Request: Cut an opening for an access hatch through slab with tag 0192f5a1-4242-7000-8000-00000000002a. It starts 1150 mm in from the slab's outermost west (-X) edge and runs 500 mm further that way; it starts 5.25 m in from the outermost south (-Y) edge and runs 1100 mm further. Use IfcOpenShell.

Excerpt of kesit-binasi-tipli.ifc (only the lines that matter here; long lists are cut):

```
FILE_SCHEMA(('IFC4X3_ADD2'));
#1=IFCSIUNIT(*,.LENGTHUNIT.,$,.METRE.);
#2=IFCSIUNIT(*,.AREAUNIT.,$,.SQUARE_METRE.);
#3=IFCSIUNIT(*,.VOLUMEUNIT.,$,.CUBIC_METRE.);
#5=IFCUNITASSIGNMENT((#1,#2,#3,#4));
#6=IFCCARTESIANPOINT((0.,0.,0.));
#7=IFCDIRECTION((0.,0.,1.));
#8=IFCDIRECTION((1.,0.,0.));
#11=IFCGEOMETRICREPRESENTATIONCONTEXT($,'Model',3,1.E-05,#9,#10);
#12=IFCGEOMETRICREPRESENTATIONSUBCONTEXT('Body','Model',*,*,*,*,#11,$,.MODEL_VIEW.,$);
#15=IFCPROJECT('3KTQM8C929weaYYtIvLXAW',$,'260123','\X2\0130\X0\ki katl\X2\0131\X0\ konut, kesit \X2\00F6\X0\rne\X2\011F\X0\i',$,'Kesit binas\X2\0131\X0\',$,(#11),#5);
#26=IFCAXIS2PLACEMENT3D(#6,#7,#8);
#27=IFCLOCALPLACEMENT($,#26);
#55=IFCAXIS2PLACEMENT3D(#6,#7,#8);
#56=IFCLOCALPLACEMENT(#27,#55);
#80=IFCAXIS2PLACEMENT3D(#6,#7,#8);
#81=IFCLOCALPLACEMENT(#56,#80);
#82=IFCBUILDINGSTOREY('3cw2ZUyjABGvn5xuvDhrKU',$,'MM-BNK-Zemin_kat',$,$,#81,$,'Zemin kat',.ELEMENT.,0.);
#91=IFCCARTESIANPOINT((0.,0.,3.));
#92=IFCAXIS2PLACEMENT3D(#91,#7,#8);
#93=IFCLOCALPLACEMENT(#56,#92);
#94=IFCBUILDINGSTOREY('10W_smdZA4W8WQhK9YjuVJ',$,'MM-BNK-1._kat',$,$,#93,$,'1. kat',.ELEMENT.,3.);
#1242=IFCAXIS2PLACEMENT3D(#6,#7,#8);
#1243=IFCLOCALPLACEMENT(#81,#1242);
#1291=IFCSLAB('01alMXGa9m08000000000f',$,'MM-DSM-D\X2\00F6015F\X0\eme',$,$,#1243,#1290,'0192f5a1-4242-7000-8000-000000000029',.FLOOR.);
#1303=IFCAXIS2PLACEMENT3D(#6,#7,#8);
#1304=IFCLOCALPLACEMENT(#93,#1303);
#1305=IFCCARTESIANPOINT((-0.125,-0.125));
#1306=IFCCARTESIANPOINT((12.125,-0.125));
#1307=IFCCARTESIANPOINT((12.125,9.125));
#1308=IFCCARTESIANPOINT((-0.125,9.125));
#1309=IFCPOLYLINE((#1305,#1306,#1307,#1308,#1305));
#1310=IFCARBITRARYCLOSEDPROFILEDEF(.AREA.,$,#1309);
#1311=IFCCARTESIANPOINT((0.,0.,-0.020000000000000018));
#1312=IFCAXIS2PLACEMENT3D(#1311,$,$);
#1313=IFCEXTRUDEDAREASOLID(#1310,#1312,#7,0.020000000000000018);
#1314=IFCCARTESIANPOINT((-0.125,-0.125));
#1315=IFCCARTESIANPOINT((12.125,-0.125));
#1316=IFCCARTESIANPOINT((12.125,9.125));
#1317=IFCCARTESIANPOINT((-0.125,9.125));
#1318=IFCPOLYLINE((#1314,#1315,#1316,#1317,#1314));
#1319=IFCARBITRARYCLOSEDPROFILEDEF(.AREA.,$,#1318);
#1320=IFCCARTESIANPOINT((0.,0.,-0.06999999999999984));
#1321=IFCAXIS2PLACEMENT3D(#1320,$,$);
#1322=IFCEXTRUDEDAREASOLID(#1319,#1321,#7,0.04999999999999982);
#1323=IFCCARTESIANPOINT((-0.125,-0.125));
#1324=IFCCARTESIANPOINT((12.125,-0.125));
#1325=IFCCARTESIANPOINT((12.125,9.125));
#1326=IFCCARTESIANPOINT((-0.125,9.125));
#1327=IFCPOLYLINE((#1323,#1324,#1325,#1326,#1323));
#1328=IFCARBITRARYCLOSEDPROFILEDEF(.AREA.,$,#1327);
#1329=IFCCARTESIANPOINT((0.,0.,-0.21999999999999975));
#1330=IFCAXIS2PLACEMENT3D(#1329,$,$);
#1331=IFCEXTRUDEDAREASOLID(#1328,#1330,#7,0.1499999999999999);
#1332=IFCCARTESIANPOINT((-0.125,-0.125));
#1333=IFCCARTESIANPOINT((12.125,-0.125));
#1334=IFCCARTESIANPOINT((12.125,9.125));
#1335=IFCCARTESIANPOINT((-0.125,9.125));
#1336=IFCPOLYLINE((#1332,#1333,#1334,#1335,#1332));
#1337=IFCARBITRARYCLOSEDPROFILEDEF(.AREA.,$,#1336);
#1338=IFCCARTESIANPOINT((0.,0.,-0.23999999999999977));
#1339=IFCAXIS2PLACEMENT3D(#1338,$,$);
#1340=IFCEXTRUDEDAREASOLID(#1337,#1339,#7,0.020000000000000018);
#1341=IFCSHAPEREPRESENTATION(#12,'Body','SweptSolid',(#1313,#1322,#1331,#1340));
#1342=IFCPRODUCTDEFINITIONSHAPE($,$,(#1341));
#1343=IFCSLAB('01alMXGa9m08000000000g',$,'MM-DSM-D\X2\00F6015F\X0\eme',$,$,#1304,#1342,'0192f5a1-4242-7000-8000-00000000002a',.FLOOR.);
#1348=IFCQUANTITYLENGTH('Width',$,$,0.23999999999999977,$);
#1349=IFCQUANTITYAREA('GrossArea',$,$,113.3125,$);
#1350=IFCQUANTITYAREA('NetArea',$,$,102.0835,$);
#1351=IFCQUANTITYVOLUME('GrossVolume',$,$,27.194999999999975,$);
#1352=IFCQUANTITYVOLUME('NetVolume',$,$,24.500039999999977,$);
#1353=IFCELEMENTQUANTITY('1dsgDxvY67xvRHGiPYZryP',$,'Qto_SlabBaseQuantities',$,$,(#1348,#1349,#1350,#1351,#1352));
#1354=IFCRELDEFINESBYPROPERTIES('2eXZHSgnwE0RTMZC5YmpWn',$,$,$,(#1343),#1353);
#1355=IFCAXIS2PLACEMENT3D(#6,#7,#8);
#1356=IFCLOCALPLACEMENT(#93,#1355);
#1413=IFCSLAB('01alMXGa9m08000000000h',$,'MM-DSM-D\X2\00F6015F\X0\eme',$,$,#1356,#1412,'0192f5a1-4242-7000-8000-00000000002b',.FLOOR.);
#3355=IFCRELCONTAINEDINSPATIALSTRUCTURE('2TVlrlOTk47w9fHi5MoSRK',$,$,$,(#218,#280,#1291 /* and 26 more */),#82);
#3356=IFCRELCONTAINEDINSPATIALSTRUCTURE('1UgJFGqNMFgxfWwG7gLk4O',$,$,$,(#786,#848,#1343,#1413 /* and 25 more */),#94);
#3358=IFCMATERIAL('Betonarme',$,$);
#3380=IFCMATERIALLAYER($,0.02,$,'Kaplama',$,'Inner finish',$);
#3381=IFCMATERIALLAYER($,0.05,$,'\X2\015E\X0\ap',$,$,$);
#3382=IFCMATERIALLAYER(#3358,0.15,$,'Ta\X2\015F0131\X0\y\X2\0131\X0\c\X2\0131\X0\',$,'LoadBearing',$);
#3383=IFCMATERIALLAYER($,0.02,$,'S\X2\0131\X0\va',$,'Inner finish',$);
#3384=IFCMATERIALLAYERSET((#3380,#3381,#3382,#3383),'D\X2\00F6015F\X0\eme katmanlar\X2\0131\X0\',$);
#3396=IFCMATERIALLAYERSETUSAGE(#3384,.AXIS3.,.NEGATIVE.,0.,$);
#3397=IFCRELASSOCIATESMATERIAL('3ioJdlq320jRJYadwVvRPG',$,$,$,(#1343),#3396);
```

```python
import numpy as np
import ifcopenshell
import ifcopenshell.api.feature
import ifcopenshell.api.geometry
import ifcopenshell.api.pset
import ifcopenshell.api.root
import ifcopenshell.geom
import ifcopenshell.util.element
import ifcopenshell.util.placement
import ifcopenshell.util.representation
import ifcopenshell.util.shape
import ifcopenshell.util.unit

model = ifcopenshell.open("kesit-binasi-tipli.ifc")
unit_scale = ifcopenshell.util.unit.calculate_unit_scale(model)
area_scale = ifcopenshell.util.unit.calculate_unit_scale(model, "AREAUNIT")
volume_scale = ifcopenshell.util.unit.calculate_unit_scale(model, "VOLUMEUNIT")
settings = ifcopenshell.geom.settings()


def volume(element):
    """Net volume in cubic metres, openings subtracted."""
    shape = ifcopenshell.geom.create_shape(settings, element)
    return ifcopenshell.util.shape.get_volume(shape.geometry)


slab = model.by_guid("01alMXGa9m08000000000g")
before = volume(slab)

# Extent in the slab's own axes, in metres. The edges named are its -X and -Y sides.
slab_shape = ifcopenshell.geom.create_shape(settings, slab)
vertices = ifcopenshell.util.shape.get_vertices(slab_shape.geometry)
x_min, y_min, bottom = vertices.min(axis=0)
top = vertices[:, 2].max()

opening = ifcopenshell.api.root.create_entity(model, ifc_class="IfcOpeningElement", name="Access hatch opening", predefined_type="OPENING")
context = ifcopenshell.util.representation.get_context(model, "Model", "Body", "MODEL_VIEW")
width, depth = 0.5, 1.1
outline = [(0.0, 0.0), (width, 0.0), (width, depth), (0.0, depth), (0.0, 0.0)]
# Overshoot both faces by 50 mm so the cut is clean.
shape = ifcopenshell.api.geometry.add_slab_representation(
    model, context=context, depth=top - bottom + 0.1, polyline=outline
)
ifcopenshell.api.geometry.assign_representation(model, product=opening, representation=shape)

matrix = ifcopenshell.util.placement.get_local_placement(slab.ObjectPlacement)
matrix[:, 3] = matrix @ np.append(np.array([x_min + 1.15, y_min + 5.25, bottom - 0.05]) / unit_scale, 1.0)
ifcopenshell.api.geometry.edit_object_placement(model, product=opening, matrix=matrix, is_si=False)
ifcopenshell.api.feature.add_feature(model, feature=opening, element=slab)

after = volume(slab)

# Update the slab's stored quantities.
qto = model.by_id(ifcopenshell.util.element.get_pset(slab, "Qto_SlabBaseQuantities", should_inherit=False)["id"])
ifcopenshell.api.pset.edit_qto(model, qto=qto, properties={
    "NetArea": after / (top - bottom) / area_scale,
    "NetVolume": after / volume_scale,
})

print(f"slab volume {before:.3f} -> {after:.3f} m3")

model.write("kesit-binasi-tipli_v2.ifc")
```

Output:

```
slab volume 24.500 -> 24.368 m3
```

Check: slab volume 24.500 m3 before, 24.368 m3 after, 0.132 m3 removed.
